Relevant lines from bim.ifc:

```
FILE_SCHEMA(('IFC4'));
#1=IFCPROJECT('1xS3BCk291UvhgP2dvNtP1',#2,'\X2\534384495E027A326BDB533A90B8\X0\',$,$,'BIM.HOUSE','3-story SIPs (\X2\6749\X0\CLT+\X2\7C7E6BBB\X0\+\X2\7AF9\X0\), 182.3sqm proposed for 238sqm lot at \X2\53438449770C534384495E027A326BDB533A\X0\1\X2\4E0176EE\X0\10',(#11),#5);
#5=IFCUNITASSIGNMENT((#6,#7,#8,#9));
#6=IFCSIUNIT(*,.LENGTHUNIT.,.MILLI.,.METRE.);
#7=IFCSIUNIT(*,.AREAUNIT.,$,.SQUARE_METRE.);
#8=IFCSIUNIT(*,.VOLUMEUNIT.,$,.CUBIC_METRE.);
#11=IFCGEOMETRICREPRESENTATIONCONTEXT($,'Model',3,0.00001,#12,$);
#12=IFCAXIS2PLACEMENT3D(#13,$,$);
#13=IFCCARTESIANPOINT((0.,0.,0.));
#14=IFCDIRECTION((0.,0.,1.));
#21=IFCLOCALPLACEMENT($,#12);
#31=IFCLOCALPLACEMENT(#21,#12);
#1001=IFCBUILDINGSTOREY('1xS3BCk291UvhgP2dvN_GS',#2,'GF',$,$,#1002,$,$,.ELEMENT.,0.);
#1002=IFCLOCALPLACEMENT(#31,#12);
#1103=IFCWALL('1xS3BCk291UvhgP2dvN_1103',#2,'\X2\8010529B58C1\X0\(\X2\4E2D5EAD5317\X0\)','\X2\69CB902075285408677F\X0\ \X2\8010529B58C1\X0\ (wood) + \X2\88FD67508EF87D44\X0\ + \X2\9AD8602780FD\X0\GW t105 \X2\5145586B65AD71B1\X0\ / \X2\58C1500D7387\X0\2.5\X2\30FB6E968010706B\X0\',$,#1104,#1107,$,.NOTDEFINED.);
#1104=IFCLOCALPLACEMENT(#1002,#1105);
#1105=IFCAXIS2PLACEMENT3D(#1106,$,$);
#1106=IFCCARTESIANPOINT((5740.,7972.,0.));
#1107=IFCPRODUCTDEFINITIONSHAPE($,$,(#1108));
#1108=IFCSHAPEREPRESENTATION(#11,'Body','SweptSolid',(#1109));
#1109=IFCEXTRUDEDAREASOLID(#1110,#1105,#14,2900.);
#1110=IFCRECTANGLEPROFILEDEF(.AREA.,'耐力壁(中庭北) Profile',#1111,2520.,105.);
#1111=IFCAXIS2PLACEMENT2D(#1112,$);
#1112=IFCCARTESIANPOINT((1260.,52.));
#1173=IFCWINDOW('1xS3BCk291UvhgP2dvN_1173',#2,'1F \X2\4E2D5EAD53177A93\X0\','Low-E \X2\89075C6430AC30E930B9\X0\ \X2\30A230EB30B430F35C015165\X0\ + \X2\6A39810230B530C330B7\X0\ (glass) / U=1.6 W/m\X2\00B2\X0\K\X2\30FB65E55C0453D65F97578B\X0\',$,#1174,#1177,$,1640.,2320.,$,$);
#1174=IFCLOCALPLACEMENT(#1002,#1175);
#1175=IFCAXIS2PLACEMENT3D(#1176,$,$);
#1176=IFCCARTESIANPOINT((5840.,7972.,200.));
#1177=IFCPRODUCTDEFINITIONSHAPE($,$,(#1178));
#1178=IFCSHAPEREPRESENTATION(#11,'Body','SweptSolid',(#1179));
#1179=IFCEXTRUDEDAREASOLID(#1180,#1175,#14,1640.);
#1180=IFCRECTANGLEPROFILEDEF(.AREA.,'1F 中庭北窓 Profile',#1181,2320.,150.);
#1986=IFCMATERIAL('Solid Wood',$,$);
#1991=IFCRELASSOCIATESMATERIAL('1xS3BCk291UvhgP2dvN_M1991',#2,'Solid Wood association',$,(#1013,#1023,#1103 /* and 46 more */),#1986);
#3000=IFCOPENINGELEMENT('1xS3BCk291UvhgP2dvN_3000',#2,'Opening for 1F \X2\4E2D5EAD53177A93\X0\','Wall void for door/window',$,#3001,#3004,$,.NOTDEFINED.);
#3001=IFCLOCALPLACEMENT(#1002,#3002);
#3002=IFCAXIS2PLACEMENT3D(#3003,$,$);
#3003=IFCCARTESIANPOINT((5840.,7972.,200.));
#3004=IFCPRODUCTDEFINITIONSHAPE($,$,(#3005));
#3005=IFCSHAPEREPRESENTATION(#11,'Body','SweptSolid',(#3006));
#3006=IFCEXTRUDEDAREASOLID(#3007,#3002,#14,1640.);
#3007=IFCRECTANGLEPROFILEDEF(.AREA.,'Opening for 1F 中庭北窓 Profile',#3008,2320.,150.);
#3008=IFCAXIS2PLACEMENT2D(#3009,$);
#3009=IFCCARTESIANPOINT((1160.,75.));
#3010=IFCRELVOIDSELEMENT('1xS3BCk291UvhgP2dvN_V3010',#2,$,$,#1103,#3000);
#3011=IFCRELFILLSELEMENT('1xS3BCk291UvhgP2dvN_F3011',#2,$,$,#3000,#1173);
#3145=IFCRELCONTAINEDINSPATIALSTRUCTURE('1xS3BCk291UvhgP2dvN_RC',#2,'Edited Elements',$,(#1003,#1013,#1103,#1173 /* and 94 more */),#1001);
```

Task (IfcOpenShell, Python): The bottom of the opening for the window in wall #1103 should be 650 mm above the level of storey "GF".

```python
import numpy as np
import ifcopenshell
import ifcopenshell.api.geometry
import ifcopenshell.geom
import ifcopenshell.util.element
import ifcopenshell.util.placement
import ifcopenshell.util.shape
import ifcopenshell.util.unit

model = ifcopenshell.open("bim.ifc")
unit_scale = ifcopenshell.util.unit.calculate_unit_scale(model)

window = model.by_guid("1xS3BCk291UvhgP2dvN_1173")
opening = window.FillsVoids[0].RelatingOpeningElement
storey = ifcopenshell.util.element.get_container(window, ifc_class="IfcBuildingStorey")
level = ifcopenshell.util.placement.get_local_placement(storey.ObjectPlacement)[2, 3]

# The opening's origin need not be at the sill, so measure its lowest point.
shape = ifcopenshell.geom.create_shape(ifcopenshell.geom.settings(), opening)
bottom = ifcopenshell.util.shape.get_shape_bottom_elevation(shape, shape.geometry) / unit_scale
dz = level + 0.65 / unit_scale - bottom

shift = np.array([0.0, 0.0, dz])
# The window is not placed relative to its opening, so move both.
for product in (opening, window):
    matrix = ifcopenshell.util.placement.get_local_placement(product.ObjectPlacement)
    matrix[:3, 3] += shift
    ifcopenshell.api.geometry.edit_object_placement(model, product=product, matrix=matrix, is_si=False)

print(f"moved by {dz * unit_scale:+.3f} m")

model.write("bim_rev.ifc")
```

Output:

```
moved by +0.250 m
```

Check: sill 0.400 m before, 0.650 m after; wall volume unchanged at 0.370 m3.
